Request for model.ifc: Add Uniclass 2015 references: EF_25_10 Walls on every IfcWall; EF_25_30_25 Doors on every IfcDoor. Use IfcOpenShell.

First a look at what the model holds.

```python
import ifcopenshell

model = ifcopenshell.open("model.ifc")
print(model.schema)
print("classifications:", [c.Name for c in model.by_type("IfcClassification")])
for ifc_class in ("IfcDoor", "IfcRoof", "IfcStair", "IfcWall", "IfcWindow"):
    print(ifc_class, len(model.by_type(ifc_class)))
```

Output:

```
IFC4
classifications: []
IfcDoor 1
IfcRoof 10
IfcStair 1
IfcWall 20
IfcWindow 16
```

```python
import ifcopenshell
import ifcopenshell.api.classification

model = ifcopenshell.open("model.ifc")

system = ifcopenshell.api.classification.add_classification(model, classification="Uniclass 2015")

codes = {
    "IfcWall": ("EF_25_10", "Walls"),
    "IfcDoor": ("EF_25_30_25", "Doors"),
}
for ifc_class, (code, name) in codes.items():
    products = model.by_type(ifc_class)
    ifcopenshell.api.classification.add_reference(
        model, products=products, classification=system, identification=code, name=name
    )
    print(code, len(products))

model.write("model_rev.ifc")
```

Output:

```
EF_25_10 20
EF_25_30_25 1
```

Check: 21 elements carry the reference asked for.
